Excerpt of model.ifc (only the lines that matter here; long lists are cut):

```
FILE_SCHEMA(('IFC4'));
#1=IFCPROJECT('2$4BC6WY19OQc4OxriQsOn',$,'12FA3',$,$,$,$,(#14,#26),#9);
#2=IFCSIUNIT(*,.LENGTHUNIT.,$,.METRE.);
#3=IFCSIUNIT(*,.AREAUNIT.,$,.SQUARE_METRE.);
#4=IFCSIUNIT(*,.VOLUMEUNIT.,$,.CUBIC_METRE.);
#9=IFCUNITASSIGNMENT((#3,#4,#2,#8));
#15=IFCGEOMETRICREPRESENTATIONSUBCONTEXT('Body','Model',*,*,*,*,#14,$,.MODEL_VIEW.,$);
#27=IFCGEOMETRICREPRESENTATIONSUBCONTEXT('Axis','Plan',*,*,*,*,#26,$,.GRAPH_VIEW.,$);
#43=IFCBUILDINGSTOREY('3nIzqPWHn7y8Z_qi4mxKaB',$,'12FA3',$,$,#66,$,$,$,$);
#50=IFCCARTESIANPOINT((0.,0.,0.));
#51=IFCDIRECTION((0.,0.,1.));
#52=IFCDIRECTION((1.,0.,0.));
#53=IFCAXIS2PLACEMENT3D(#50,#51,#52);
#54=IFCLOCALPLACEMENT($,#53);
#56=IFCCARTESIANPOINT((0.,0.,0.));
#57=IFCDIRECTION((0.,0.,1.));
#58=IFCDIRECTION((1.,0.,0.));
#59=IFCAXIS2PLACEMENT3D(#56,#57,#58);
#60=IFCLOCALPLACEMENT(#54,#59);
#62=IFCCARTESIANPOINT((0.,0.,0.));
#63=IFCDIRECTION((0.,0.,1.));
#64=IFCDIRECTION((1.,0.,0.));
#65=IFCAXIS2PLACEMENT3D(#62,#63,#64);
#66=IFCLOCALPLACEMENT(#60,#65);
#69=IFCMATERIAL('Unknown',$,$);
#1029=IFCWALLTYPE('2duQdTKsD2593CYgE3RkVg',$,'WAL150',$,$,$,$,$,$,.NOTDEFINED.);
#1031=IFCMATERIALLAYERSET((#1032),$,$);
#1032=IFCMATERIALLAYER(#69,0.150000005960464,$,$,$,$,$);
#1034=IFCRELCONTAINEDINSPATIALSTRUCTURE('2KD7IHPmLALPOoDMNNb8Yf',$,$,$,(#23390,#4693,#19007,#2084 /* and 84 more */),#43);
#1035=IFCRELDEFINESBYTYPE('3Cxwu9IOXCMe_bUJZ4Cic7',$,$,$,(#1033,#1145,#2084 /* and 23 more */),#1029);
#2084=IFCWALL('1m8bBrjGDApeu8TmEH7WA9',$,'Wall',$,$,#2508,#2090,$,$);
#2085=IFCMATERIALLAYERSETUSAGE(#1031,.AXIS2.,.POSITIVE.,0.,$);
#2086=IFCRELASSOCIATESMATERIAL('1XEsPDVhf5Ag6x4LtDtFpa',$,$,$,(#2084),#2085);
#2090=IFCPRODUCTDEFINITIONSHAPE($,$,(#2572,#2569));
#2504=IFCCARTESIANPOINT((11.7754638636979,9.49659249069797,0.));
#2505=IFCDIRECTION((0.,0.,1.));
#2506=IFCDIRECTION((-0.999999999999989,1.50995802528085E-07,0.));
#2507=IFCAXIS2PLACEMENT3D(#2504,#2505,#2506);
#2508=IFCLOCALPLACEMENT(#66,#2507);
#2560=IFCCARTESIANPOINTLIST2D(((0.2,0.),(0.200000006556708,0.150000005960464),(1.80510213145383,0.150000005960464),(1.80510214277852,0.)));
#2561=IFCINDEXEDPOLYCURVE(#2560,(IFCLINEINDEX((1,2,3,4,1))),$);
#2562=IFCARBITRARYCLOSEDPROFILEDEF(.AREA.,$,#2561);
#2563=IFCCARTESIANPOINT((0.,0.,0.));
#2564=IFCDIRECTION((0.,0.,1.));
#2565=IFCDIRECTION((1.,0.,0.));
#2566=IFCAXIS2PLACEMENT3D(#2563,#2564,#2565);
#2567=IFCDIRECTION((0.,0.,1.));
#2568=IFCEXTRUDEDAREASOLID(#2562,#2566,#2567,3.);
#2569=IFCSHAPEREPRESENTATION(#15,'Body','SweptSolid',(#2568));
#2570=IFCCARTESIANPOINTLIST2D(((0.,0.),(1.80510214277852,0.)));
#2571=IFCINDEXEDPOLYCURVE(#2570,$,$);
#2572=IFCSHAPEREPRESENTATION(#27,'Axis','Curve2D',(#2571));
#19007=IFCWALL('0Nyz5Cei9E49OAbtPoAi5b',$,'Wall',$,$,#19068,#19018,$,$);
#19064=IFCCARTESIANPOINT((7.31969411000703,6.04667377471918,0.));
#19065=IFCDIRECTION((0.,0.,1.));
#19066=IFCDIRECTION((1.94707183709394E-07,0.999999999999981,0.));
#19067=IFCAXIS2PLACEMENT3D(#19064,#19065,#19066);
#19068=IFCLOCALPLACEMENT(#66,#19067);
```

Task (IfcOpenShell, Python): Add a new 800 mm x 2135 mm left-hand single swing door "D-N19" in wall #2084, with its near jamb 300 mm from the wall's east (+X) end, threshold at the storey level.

```python
import numpy as np
import ifcopenshell
import ifcopenshell.api.feature
import ifcopenshell.api.geometry
import ifcopenshell.api.root
import ifcopenshell.api.spatial
import ifcopenshell.geom
import ifcopenshell.util.element
import ifcopenshell.util.placement
import ifcopenshell.util.representation
import ifcopenshell.util.shape
import ifcopenshell.util.unit

model = ifcopenshell.open("model.ifc")
unit_scale = ifcopenshell.util.unit.calculate_unit_scale(model)
settings = ifcopenshell.geom.settings()


def volume(element):
    """Net volume in cubic metres, openings subtracted."""
    shape = ifcopenshell.geom.create_shape(settings, element)
    return ifcopenshell.util.shape.get_volume(shape.geometry)


wall = model.by_guid("1m8bBrjGDApeu8TmEH7WA9")
storey = ifcopenshell.util.element.get_container(wall, ifc_class="IfcBuildingStorey")
context = ifcopenshell.util.representation.get_context(model, "Model", "Body", "MODEL_VIEW")
before = volume(wall)

width, height, from_end, sill = 0.8, 2.135, 0.3, 0.0  # metres

# The wall runs along its own X axis, and the end named is its -X end.
wall_shape = ifcopenshell.geom.create_shape(settings, wall)
x, y, z = ifcopenshell.util.shape.get_vertices(wall_shape.geometry).T
start = x.min() + from_end
face, thickness = float(y.min()), float(y.max() - y.min())
wall_matrix = ifcopenshell.util.placement.get_local_placement(wall.ObjectPlacement)
level = ifcopenshell.util.placement.get_local_placement(storey.ObjectPlacement)[2, 3]


def in_wall(x, y):
    """Placement at x, y metres in the wall's axes, at sill height."""
    matrix = wall_matrix.copy()
    matrix[:, 3] = wall_matrix @ np.array([x / unit_scale, y / unit_scale, 0.0, 1.0])
    matrix[2, 3] = level + sill / unit_scale
    return matrix


# Opening: a box that overshoots both wall faces by 50 mm.
opening = ifcopenshell.api.root.create_entity(model, ifc_class="IfcOpeningElement", predefined_type="OPENING")
box = ifcopenshell.api.geometry.add_wall_representation(
    model, context=context, length=width, height=height, thickness=thickness + 0.1
)
ifcopenshell.api.geometry.assign_representation(model, product=opening, representation=box)
ifcopenshell.api.geometry.edit_object_placement(model, product=opening, matrix=in_wall(start, face - 0.05), is_si=False)
ifcopenshell.api.feature.add_feature(model, feature=opening, element=wall)

door = ifcopenshell.api.root.create_entity(model, ifc_class="IfcDoor", name="D-N19", predefined_type="DOOR")
door.OverallWidth, door.OverallHeight = width / unit_scale, height / unit_scale
door.OperationType = "SINGLE_SWING_LEFT"
body = ifcopenshell.api.geometry.add_door_representation(
    model,
    context=context,
    overall_width=door.OverallWidth,
    overall_height=door.OverallHeight,
    operation_type="SINGLE_SWING_LEFT",
    lining_properties={"LiningDepth": thickness / unit_scale, "ThresholdDepth": thickness / unit_scale},
)
ifcopenshell.api.geometry.assign_representation(model, product=door, representation=body)
ifcopenshell.api.spatial.assign_container(model, products=[door], relating_structure=storey)
ifcopenshell.api.feature.add_filling(model, opening=opening, element=door)

# The lining spans the wall, so the door starts at the wall face.
ifcopenshell.api.geometry.edit_object_placement(model, product=door, matrix=in_wall(start, face), is_si=False)

after = volume(wall)

print(f"wall volume {before:.3f} -> {after:.3f} m3")

model.write("model_updated.ifc")
```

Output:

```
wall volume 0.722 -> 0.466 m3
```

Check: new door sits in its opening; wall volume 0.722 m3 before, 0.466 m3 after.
